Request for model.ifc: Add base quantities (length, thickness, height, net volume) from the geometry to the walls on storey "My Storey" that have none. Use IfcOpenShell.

First a look at what the model holds.

```python
import ifcopenshell
import ifcopenshell.util.element
import ifcopenshell.util.unit

model = ifcopenshell.open("model.ifc")
print(model.schema)
for unit_type in ("LENGTHUNIT", "AREAUNIT", "VOLUMEUNIT"):
    print(unit_type, ifcopenshell.util.unit.calculate_unit_scale(model, unit_type))
storey = next(s for s in model.by_type("IfcBuildingStorey") if s.Name == "My Storey")
walls = [e for e in ifcopenshell.util.element.get_decomposition(storey) if e.is_a("IfcWall")]
for e in sorted(walls, key=lambda e: e.id()):
    print(e.id(), e.is_a(), e.Name, list(ifcopenshell.util.element.get_psets(e, qtos_only=True)), sep=" | ")
```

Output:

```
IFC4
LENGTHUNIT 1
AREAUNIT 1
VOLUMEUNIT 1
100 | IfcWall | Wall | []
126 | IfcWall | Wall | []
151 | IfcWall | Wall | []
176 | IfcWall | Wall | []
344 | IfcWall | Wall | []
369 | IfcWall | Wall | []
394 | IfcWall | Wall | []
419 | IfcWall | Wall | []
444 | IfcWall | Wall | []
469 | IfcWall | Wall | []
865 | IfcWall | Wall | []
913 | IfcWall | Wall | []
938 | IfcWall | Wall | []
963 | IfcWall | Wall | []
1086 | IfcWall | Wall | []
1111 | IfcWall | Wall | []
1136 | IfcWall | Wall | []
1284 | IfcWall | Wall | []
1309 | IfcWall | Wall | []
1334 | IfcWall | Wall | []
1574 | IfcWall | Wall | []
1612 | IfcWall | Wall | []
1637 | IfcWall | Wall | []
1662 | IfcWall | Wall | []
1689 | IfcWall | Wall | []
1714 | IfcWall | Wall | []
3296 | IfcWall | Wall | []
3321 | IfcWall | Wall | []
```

```python
import ifcopenshell
import ifcopenshell.api.pset
import ifcopenshell.geom
import ifcopenshell.util.element
import ifcopenshell.util.shape
import ifcopenshell.util.unit

model = ifcopenshell.open("model.ifc")
unit_scale = ifcopenshell.util.unit.calculate_unit_scale(model)
volume_scale = ifcopenshell.util.unit.calculate_unit_scale(model, "VOLUMEUNIT")
settings = ifcopenshell.geom.settings()

storey = next(s for s in model.by_type("IfcBuildingStorey") if s.Name == "My Storey")
walls = [e for e in ifcopenshell.util.element.get_decomposition(storey) if e.is_a("IfcWall")]

for e in sorted(walls, key=lambda e: e.id()):
    if ifcopenshell.util.element.get_psets(e, qtos_only=True, should_inherit=False):
        continue
    # Geometry comes back in metres, in the element's own axes.
    shape = ifcopenshell.geom.create_shape(settings, e)
    values = {
        "Length": ifcopenshell.util.shape.get_x(shape.geometry) / unit_scale,
        "Width": ifcopenshell.util.shape.get_y(shape.geometry) / unit_scale,
        "Height": ifcopenshell.util.shape.get_z(shape.geometry) / unit_scale,
        "NetVolume": ifcopenshell.util.shape.get_volume(shape.geometry) / volume_scale,
    }
    qto = ifcopenshell.api.pset.add_qto(model, product=e, name="Qto_WallBaseQuantities")
    ifcopenshell.api.pset.edit_qto(model, qto=qto, properties=values)
    print(e.id(), {k: round(v, 3) for k, v in values.items()})

model.write("model_updated.ifc")
```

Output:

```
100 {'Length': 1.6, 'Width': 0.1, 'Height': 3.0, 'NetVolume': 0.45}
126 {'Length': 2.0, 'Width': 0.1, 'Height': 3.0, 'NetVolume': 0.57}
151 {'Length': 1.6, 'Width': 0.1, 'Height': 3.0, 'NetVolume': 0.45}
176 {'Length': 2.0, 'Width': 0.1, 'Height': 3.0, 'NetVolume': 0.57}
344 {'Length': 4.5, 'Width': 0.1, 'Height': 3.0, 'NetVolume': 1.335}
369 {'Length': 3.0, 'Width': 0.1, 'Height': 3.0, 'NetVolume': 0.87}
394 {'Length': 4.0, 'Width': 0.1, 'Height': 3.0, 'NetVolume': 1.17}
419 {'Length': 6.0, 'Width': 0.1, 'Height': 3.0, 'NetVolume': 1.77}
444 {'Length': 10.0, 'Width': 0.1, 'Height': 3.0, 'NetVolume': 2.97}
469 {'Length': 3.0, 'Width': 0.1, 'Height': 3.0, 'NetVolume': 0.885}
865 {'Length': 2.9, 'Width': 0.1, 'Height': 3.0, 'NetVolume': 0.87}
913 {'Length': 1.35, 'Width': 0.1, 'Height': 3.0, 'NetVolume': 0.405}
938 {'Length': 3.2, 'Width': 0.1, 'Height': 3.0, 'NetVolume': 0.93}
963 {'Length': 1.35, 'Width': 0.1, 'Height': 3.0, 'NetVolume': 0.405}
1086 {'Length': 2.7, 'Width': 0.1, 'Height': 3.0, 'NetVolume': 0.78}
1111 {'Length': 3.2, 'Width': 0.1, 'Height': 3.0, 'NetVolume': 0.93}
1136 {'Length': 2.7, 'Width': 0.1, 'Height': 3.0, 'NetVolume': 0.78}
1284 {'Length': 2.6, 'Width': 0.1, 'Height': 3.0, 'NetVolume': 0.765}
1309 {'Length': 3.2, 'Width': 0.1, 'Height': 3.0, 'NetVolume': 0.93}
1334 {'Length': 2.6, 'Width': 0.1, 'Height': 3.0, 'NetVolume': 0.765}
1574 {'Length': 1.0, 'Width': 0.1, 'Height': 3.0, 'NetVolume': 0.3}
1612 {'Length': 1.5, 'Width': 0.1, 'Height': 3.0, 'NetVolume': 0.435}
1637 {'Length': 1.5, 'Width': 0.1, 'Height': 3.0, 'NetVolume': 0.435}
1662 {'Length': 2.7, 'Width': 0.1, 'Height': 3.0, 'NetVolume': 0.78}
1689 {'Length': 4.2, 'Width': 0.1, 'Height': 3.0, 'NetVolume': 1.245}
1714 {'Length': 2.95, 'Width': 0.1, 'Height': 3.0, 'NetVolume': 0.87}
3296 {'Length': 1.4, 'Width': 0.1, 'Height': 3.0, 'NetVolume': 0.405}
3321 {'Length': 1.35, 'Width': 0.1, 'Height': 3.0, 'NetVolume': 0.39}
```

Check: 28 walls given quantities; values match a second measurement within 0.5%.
